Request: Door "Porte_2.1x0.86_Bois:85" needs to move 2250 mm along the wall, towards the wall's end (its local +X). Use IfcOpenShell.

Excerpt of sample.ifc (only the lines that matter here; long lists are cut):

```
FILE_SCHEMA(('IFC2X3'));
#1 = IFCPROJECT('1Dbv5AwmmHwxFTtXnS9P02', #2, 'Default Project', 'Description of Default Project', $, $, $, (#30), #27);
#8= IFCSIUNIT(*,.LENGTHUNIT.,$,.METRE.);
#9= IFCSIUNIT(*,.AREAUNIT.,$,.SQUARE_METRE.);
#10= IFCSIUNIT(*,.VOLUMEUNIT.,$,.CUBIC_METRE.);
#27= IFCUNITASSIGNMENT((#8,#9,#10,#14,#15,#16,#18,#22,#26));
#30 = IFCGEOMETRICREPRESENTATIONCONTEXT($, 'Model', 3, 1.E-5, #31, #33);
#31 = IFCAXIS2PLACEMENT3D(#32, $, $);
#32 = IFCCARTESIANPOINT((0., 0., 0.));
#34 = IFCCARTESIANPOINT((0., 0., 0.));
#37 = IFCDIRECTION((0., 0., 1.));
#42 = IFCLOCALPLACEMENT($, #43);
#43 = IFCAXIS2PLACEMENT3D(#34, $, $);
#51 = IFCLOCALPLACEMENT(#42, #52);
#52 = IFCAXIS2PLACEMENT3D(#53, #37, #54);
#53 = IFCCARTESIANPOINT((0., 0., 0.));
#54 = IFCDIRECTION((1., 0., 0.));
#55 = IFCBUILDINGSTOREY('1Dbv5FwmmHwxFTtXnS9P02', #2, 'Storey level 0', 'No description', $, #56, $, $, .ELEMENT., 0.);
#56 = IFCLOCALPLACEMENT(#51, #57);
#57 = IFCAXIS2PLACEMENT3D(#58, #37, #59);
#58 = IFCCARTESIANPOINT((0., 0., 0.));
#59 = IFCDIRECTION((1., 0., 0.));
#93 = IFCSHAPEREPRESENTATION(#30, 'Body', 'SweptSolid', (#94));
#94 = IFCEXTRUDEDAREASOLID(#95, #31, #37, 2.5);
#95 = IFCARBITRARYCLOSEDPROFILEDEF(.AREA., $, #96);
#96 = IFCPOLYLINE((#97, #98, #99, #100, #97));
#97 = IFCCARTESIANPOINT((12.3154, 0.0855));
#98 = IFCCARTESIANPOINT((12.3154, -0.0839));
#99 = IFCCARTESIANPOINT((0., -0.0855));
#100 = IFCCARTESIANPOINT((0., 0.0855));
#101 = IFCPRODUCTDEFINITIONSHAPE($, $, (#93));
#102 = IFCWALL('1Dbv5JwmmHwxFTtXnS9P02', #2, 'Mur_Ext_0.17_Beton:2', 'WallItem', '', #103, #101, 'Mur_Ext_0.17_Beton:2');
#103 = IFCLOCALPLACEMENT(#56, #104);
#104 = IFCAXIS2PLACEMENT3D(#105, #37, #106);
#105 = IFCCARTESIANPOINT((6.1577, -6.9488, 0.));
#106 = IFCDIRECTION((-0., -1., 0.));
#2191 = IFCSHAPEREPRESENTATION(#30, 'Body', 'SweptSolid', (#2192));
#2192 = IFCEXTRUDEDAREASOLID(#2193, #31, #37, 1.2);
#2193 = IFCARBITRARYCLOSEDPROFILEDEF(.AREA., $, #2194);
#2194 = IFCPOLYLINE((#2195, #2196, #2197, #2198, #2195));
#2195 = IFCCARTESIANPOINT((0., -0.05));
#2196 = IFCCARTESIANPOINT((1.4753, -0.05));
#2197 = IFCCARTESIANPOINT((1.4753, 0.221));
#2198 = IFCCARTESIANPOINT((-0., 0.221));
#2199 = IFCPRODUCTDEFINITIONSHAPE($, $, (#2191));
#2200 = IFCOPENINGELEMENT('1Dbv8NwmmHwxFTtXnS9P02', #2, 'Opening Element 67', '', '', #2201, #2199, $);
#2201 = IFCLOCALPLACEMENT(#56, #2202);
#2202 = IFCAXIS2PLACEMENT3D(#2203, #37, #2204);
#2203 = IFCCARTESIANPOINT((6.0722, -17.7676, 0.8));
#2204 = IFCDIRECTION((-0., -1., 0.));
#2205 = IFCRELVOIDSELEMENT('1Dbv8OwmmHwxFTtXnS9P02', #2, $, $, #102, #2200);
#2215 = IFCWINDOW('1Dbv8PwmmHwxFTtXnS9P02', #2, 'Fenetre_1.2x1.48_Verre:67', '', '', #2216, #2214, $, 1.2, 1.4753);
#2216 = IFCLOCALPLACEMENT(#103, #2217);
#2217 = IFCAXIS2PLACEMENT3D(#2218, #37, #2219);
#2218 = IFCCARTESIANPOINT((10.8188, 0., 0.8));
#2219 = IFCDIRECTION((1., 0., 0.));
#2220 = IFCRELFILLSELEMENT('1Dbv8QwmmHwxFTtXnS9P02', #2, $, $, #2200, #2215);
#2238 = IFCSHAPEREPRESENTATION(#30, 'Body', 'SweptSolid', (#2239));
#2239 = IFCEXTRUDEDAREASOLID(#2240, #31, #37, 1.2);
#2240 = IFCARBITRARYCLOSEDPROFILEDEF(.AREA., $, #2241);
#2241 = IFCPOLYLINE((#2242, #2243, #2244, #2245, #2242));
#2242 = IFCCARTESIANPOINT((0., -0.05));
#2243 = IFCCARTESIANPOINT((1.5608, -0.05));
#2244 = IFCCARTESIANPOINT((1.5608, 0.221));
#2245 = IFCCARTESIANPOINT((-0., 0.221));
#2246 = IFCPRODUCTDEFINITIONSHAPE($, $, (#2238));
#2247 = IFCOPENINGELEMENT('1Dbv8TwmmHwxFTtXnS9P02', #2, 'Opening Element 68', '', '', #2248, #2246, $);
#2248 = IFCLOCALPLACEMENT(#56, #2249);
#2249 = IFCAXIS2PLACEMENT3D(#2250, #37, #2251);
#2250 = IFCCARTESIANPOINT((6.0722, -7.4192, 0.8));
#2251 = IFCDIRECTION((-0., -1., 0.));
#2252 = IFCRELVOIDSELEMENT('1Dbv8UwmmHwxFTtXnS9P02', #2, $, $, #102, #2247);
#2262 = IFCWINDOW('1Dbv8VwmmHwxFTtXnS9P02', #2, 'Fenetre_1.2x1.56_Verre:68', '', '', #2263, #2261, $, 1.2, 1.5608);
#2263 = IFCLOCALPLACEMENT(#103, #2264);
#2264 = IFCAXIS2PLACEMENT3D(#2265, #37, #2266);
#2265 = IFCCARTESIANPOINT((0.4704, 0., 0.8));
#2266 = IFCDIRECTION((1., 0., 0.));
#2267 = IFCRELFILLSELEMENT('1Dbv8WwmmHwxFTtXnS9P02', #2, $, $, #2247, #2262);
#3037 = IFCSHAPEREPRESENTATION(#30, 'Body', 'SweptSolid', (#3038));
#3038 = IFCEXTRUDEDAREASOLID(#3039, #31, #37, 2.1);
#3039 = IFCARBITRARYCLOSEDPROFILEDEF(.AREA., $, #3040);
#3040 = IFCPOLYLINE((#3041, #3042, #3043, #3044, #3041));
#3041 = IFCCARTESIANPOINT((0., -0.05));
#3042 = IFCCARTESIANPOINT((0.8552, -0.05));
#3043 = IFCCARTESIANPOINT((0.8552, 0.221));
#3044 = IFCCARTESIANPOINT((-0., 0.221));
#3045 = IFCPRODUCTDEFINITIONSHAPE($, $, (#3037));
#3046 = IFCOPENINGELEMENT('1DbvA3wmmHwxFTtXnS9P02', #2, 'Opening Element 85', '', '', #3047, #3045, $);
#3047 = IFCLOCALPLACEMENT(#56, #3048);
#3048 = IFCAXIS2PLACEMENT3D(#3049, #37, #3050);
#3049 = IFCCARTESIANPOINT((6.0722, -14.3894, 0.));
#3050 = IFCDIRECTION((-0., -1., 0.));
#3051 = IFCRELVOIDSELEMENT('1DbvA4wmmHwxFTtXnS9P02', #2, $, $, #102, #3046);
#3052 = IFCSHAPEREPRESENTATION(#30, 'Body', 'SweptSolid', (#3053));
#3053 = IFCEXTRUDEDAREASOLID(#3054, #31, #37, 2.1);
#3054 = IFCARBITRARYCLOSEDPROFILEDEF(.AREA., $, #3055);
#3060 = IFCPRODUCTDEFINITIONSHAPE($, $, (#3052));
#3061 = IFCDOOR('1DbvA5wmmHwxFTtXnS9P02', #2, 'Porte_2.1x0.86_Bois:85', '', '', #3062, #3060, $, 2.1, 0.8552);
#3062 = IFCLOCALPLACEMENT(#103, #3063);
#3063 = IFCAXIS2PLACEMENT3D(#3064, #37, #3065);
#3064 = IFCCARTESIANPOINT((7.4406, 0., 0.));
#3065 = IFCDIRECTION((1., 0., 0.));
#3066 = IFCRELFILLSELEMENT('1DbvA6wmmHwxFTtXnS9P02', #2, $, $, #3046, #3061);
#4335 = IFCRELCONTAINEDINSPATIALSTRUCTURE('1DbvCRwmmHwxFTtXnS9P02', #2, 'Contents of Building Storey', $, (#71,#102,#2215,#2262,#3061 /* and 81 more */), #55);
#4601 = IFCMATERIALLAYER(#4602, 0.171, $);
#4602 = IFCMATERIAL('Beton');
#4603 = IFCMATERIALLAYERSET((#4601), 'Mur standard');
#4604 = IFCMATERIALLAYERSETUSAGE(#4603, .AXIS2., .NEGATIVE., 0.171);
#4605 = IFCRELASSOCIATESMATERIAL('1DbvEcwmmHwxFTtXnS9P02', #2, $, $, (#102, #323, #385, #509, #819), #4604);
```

```python
import ifcopenshell
import ifcopenshell.api.geometry
import ifcopenshell.util.placement
import ifcopenshell.util.unit

model = ifcopenshell.open("sample.ifc")
unit_scale = ifcopenshell.util.unit.calculate_unit_scale(model)

door = model.by_guid("1DbvA5wmmHwxFTtXnS9P02")
opening = door.FillsVoids[0].RelatingOpeningElement
wall = opening.VoidsElements[0].RelatingBuildingElement

wall_matrix = ifcopenshell.util.placement.get_local_placement(wall.ObjectPlacement)
shift = wall_matrix[:3, 0] * 2.25 / unit_scale
before = ifcopenshell.util.placement.get_local_placement(door.ObjectPlacement)[:3, 3].copy()

# The door is not placed relative to its opening, so move both.
for product in (opening, door):
    matrix = ifcopenshell.util.placement.get_local_placement(product.ObjectPlacement)
    matrix[:3, 3] += shift
    ifcopenshell.api.geometry.edit_object_placement(model, product=product, matrix=matrix, is_si=False)

after = ifcopenshell.util.placement.get_local_placement(door.ObjectPlacement)[:3, 3]
print("door moved by", (after - before).round(3) + 0.0)

model.write("sample_updated.ifc")
```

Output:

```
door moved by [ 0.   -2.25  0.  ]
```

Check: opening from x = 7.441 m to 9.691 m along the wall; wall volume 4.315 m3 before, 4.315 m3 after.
